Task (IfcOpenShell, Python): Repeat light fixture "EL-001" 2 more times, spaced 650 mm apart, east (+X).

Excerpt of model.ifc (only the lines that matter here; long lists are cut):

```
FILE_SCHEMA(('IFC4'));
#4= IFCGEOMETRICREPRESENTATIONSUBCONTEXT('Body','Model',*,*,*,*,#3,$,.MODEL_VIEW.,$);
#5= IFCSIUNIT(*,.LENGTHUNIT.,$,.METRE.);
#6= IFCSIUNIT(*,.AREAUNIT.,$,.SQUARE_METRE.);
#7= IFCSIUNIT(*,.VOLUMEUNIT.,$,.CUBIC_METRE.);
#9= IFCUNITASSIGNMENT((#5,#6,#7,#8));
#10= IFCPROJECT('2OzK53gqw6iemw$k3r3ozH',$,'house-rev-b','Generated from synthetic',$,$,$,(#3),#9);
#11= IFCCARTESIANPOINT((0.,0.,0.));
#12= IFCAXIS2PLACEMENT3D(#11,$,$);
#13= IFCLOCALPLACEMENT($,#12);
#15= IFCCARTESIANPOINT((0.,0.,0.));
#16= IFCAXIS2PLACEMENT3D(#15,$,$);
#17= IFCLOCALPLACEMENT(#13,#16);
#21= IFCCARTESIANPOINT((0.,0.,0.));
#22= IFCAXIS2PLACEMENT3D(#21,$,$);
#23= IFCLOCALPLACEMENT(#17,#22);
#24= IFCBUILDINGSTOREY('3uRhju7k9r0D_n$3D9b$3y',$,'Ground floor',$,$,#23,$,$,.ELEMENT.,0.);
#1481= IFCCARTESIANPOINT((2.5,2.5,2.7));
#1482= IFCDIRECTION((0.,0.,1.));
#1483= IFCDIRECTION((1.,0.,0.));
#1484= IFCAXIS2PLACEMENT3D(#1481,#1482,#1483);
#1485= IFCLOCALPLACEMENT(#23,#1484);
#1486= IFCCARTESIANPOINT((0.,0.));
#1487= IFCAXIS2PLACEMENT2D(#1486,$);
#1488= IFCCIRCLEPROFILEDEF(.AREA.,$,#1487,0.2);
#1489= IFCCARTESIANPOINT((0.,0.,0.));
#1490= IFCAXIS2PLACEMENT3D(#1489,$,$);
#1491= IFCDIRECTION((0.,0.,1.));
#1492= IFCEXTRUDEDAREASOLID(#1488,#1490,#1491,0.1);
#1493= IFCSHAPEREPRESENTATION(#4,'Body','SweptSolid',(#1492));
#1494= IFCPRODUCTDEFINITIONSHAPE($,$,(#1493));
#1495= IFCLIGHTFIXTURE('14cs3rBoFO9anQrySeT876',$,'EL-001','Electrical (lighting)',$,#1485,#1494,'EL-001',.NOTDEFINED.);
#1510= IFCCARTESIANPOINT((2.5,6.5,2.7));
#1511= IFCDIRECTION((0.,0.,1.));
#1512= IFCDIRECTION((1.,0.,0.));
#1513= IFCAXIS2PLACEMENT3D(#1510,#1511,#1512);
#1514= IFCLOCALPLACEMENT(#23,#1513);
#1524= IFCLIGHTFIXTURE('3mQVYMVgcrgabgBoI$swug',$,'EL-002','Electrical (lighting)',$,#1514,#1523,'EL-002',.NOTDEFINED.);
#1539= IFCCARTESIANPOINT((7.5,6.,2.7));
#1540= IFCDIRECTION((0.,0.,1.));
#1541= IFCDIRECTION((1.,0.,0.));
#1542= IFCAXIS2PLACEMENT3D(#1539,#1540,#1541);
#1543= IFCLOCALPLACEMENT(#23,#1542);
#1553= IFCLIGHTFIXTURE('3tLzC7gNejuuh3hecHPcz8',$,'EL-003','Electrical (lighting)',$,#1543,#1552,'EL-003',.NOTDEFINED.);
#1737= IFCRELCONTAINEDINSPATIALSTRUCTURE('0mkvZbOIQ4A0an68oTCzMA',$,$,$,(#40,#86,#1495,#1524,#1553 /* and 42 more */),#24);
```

```python
import numpy as np
import ifcopenshell
import ifcopenshell.api.geometry
import ifcopenshell.api.root
import ifcopenshell.util.element
import ifcopenshell.util.placement
import ifcopenshell.util.unit

model = ifcopenshell.open("model.ifc")
unit_scale = ifcopenshell.util.unit.calculate_unit_scale(model)

source = model.by_guid("14cs3rBoFO9anQrySeT876")
base = ifcopenshell.util.placement.get_local_placement(source.ObjectPlacement)
step = np.array([1.0, 0.0, 0.0]) * 0.65 / unit_scale

for i in range(1, 3):
    copy = ifcopenshell.api.root.copy_class(model, product=source)
    copy.Representation = ifcopenshell.util.element.copy_deep(
        model, source.Representation, exclude=["IfcGeometricRepresentationContext", "IfcRepresentationMap"]
    )
    copy.Tag = None
    matrix = base.copy()
    matrix[:3, 3] += i * step
    print("added at", matrix[:3, 3].round(3) + 0.0)
    ifcopenshell.api.geometry.edit_object_placement(model, product=copy, matrix=matrix, is_si=False)

model.write("model_rev.ifc")
```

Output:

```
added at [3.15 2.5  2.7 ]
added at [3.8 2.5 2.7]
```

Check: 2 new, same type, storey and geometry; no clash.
